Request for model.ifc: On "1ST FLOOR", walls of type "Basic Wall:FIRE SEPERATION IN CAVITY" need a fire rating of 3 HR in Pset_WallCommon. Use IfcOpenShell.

First a look at what the model holds.

```python
import ifcopenshell
import ifcopenshell.util.element

model = ifcopenshell.open("model.ifc")
print(model.schema)
storey = next(s for s in model.by_type("IfcBuildingStorey") if s.Name == "1ST FLOOR")
walls = [e for e in ifcopenshell.util.element.get_decomposition(storey) if e.is_a("IfcWall")]
seen = {}
for e in walls:
    element_type = ifcopenshell.util.element.get_type(e)
    key = (element_type.Name if element_type != e and element_type else None, ifcopenshell.util.element.get_pset(e, "Pset_WallCommon", "FireRating"))
    seen[key] = seen.get(key, 0) + 1
for (name, value), count in sorted(seen.items(), key=str):
    print(count, "x", name, "|", value)
```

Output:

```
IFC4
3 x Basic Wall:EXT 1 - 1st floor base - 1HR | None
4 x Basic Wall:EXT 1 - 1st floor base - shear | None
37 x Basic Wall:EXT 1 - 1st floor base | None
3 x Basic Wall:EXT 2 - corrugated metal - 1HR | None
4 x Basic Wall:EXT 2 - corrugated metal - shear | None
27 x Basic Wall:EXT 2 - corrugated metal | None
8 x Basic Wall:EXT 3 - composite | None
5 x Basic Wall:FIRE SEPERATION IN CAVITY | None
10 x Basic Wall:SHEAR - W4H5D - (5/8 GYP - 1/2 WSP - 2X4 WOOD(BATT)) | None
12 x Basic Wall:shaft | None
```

```python
import ifcopenshell
import ifcopenshell.api.pset
import ifcopenshell.util.element

model = ifcopenshell.open("model.ifc")

storey = next(s for s in model.by_type("IfcBuildingStorey") if s.Name == "1ST FLOOR")
walls = [e for e in ifcopenshell.util.element.get_decomposition(storey) if e.is_a("IfcWall")]

count = 0
for e in walls:
    element_type = ifcopenshell.util.element.get_type(e)
    if element_type in (None, e) or element_type.Name != "Basic Wall:FIRE SEPERATION IN CAVITY":
        continue
    # add_pset returns the element's existing set when there is one.
    pset = ifcopenshell.api.pset.add_pset(model, product=e, name="Pset_WallCommon")
    ifcopenshell.api.pset.edit_pset(model, pset=pset, properties={"FireRating": "3 HR"})
    count += 1

print(count, "walls updated")

model.write("model_v2.ifc")
```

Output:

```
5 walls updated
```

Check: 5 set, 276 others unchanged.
